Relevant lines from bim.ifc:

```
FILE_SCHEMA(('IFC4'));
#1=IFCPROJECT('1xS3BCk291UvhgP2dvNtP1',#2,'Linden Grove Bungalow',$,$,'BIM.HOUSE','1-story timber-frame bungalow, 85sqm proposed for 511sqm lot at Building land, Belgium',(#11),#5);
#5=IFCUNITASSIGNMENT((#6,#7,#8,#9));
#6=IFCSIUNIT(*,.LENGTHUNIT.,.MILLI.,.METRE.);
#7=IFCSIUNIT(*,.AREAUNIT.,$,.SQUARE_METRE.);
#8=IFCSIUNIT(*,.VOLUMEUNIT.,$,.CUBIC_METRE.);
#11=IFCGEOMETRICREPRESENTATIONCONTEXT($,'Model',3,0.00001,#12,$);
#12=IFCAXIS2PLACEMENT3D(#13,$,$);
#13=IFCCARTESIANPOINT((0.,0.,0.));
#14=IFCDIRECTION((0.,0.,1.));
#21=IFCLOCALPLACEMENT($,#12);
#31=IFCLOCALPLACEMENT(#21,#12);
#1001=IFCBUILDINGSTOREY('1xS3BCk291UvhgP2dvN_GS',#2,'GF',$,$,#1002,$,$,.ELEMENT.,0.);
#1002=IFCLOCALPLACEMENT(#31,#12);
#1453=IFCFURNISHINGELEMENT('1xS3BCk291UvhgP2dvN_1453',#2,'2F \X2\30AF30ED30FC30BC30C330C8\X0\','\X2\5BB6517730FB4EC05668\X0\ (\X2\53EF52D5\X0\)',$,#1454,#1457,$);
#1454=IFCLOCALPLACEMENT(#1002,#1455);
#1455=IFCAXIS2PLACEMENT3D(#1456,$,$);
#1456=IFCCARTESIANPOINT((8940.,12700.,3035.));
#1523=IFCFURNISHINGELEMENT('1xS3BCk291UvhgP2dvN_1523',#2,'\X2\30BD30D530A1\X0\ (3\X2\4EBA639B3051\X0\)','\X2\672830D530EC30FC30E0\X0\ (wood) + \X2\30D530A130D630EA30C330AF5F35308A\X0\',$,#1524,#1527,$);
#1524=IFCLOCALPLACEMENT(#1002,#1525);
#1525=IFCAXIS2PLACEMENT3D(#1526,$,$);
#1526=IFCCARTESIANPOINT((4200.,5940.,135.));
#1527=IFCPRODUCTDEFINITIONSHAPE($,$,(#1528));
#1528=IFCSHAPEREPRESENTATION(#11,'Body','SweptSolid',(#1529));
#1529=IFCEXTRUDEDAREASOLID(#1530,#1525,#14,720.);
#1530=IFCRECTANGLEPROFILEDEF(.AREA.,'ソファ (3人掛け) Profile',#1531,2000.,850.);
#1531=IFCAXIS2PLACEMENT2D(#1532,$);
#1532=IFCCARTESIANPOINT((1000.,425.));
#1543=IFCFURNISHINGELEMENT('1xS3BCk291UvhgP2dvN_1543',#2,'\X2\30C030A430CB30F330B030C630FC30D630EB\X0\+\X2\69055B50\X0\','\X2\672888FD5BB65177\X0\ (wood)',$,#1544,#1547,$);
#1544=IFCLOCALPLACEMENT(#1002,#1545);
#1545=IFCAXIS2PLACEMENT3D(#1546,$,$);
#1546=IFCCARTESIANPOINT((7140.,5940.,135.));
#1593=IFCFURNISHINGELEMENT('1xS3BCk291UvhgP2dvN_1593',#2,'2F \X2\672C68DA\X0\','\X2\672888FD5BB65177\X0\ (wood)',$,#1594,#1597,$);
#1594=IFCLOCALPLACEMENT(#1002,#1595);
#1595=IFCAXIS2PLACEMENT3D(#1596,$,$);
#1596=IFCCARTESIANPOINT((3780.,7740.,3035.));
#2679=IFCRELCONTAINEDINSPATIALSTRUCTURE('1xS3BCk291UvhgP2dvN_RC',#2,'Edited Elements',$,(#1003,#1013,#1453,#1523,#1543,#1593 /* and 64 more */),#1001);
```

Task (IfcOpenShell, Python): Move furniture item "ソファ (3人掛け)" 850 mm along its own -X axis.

```python
import ifcopenshell
import ifcopenshell.api.geometry
import ifcopenshell.util.placement

model = ifcopenshell.open("bim.ifc")

item = model.by_guid("1xS3BCk291UvhgP2dvN_1523")
matrix = ifcopenshell.util.placement.get_local_placement(item.ObjectPlacement)
matrix[:3, 3] -= matrix[:3, 0] * 850.0
ifcopenshell.api.geometry.edit_object_placement(model, product=item, matrix=matrix, is_si=False)

print(ifcopenshell.util.placement.get_local_placement(item.ObjectPlacement).round(3) + 0.0)

model.write("bim_updated.ifc")
```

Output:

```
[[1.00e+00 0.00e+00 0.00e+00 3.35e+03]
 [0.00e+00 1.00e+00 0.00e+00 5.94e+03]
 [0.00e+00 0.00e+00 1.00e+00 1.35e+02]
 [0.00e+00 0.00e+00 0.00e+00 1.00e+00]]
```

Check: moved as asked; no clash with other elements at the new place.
